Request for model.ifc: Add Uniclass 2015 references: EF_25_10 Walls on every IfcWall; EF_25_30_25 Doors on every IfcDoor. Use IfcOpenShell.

First a look at what the model holds.

```python
import ifcopenshell

model = ifcopenshell.open("model.ifc")
print(model.schema)
print("classifications:", [c.Name for c in model.by_type("IfcClassification")])
for ifc_class in ("IfcDoor", "IfcRoof", "IfcStair", "IfcWall", "IfcWindow"):
    print(ifc_class, len(model.by_type(ifc_class)))
```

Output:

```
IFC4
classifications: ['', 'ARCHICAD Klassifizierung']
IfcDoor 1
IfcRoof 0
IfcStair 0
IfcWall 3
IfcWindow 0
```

```python
import ifcopenshell
import ifcopenshell.api.classification

model = ifcopenshell.open("model.ifc")

system = ifcopenshell.api.classification.add_classification(model, classification="Uniclass 2015")

codes = {
    "IfcWall": ("EF_25_10", "Walls"),
    "IfcDoor": ("EF_25_30_25", "Doors"),
}
for ifc_class, (code, name) in codes.items():
    products = model.by_type(ifc_class)
    ifcopenshell.api.classification.add_reference(
        model, products=products, classification=system, identification=code, name=name
    )
    print(code, len(products))

model.write("model_edited.ifc")
```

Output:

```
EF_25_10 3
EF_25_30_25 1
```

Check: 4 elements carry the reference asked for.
